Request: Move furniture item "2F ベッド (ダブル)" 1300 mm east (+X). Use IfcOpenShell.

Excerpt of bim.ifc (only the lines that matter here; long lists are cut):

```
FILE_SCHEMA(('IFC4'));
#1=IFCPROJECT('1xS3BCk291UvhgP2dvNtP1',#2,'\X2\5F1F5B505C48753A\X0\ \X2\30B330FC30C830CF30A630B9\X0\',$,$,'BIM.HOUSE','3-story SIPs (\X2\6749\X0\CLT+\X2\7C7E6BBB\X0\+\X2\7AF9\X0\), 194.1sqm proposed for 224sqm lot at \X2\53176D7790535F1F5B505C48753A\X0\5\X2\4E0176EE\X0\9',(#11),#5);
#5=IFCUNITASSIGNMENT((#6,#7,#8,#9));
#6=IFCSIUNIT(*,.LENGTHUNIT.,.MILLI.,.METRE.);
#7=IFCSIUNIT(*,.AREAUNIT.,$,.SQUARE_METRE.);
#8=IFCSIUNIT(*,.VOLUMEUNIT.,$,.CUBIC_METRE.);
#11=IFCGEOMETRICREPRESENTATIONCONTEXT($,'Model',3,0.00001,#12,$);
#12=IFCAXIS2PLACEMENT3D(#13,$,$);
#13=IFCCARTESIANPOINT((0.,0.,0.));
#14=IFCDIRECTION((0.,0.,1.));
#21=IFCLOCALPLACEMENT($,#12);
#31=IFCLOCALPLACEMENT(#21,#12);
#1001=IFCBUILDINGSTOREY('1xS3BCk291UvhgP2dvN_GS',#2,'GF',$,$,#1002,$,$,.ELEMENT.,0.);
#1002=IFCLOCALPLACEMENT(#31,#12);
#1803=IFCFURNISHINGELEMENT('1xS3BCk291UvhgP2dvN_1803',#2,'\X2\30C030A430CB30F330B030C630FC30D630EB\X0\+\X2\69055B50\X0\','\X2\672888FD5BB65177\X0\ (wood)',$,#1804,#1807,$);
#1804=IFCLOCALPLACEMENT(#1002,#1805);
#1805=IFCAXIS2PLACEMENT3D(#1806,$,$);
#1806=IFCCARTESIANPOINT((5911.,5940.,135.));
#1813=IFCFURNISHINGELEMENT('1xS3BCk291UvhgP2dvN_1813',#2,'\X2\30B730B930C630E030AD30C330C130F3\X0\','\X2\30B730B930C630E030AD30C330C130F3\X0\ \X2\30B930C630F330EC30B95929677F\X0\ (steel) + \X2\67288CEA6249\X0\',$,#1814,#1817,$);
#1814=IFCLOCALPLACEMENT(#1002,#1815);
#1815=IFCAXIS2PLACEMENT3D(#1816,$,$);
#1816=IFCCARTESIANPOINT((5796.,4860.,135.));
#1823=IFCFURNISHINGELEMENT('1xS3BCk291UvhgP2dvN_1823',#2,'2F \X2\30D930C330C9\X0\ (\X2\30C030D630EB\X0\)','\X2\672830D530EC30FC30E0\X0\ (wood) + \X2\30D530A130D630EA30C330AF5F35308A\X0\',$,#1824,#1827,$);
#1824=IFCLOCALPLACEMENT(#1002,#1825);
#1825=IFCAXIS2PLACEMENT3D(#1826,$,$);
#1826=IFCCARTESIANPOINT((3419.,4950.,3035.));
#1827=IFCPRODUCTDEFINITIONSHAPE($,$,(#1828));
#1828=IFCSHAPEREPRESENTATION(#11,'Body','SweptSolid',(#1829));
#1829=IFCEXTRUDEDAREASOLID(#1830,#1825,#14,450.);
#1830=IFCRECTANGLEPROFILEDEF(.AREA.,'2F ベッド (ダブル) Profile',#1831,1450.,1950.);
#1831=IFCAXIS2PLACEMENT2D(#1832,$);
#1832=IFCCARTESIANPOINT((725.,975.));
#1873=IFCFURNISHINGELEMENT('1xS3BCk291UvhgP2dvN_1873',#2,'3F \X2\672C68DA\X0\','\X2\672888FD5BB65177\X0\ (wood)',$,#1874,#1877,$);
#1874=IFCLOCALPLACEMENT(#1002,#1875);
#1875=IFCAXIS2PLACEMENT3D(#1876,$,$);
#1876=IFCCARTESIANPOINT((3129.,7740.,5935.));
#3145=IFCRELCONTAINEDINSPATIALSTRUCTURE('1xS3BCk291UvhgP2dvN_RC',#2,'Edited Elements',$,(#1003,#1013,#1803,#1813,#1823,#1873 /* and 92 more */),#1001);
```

```python
import ifcopenshell
import ifcopenshell.api.geometry
import ifcopenshell.util.placement
import ifcopenshell.util.unit

model = ifcopenshell.open("bim.ifc")
unit_scale = ifcopenshell.util.unit.calculate_unit_scale(model)

item = model.by_id(1823)
matrix = ifcopenshell.util.placement.get_local_placement(item.ObjectPlacement)
matrix[0, 3] += 1.3 / unit_scale
ifcopenshell.api.geometry.edit_object_placement(model, product=item, matrix=matrix, is_si=False)

print(ifcopenshell.util.placement.get_local_placement(item.ObjectPlacement).round(3) + 0.0)

model.write("bim_rev.ifc")
```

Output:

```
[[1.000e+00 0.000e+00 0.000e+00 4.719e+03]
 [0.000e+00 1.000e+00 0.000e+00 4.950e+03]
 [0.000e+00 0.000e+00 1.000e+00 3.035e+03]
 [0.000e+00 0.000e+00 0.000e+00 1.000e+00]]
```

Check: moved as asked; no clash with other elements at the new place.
